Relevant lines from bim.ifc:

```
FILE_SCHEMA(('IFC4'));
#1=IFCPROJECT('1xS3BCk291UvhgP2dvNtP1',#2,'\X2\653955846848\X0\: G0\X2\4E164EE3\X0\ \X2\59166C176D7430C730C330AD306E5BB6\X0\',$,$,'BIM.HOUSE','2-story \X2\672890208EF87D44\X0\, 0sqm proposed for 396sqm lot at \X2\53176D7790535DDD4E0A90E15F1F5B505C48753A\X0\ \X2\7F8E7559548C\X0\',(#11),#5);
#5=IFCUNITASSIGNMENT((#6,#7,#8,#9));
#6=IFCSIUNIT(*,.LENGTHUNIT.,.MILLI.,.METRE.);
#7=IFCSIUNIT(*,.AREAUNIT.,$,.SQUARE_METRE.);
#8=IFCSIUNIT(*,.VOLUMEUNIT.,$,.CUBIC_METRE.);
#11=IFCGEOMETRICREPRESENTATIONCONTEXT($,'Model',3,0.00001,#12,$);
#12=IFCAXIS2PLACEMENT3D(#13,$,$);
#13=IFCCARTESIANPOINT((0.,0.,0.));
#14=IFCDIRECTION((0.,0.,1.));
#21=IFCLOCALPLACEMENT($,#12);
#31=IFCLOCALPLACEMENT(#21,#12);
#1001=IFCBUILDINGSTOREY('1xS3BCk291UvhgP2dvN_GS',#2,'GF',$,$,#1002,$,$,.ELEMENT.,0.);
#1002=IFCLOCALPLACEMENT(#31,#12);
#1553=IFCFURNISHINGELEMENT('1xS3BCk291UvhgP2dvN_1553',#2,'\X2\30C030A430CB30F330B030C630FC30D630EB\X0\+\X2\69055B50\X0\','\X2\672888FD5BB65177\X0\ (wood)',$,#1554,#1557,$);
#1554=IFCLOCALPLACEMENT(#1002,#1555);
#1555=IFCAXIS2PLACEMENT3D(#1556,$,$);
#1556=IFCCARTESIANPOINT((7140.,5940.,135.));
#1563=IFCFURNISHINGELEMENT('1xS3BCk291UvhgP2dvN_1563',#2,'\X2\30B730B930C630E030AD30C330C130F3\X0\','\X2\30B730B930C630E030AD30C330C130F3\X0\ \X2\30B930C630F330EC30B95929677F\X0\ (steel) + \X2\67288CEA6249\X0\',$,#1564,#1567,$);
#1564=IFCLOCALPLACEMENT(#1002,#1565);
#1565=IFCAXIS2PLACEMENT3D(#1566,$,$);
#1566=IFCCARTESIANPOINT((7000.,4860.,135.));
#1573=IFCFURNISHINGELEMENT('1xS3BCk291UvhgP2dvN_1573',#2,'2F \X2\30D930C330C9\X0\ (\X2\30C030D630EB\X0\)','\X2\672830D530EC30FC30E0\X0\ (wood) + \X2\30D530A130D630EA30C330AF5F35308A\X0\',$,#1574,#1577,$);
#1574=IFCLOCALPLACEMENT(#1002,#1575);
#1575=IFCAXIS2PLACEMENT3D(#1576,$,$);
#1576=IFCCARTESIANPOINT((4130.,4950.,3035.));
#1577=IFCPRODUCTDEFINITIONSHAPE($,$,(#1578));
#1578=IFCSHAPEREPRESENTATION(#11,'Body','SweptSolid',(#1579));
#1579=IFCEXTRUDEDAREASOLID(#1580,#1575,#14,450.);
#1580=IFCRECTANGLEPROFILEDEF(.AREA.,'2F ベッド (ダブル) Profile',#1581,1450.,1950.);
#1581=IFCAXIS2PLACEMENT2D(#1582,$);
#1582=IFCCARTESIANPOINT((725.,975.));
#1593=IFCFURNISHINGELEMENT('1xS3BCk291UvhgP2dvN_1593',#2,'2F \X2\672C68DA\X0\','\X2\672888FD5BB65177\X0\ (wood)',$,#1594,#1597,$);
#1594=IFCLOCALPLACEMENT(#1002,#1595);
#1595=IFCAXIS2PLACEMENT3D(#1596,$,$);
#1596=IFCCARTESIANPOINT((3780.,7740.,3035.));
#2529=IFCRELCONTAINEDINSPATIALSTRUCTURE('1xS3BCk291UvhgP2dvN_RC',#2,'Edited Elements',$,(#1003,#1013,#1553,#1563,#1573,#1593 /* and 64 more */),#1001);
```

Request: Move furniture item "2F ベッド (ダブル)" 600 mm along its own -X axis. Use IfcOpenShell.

```python
import ifcopenshell
import ifcopenshell.api.geometry
import ifcopenshell.util.placement
import ifcopenshell.util.unit

model = ifcopenshell.open("bim.ifc")
unit_scale = ifcopenshell.util.unit.calculate_unit_scale(model)

item = model.by_guid("1xS3BCk291UvhgP2dvN_1573")
matrix = ifcopenshell.util.placement.get_local_placement(item.ObjectPlacement)
matrix[:3, 3] -= matrix[:3, 0] * 0.6 / unit_scale
ifcopenshell.api.geometry.edit_object_placement(model, product=item, matrix=matrix, is_si=False)

print(ifcopenshell.util.placement.get_local_placement(item.ObjectPlacement).round(3) + 0.0)

model.write("bim_updated.ifc")
```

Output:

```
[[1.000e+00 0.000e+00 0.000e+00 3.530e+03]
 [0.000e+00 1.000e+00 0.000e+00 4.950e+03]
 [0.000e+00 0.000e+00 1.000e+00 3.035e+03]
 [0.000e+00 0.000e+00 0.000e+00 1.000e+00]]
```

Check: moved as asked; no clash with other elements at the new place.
